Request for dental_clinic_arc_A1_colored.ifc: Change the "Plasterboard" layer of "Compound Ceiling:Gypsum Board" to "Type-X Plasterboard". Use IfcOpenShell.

First a look at what the model holds.

```python
import ifcopenshell
import ifcopenshell.util.element

model = ifcopenshell.open("dental_clinic_arc_A1_colored.ifc")
print(model.schema)
for layer_set in model.by_type("IfcMaterialLayerSet"):
    if layer_set.LayerSetName == "Compound Ceiling:Gypsum Board":
        for layer in layer_set.MaterialLayers:
            print(layer.id(), layer.Material and layer.Material.Name, layer.LayerThickness, sep=" | ")
        print(len(ifcopenshell.util.element.get_elements_by_material(model, layer_set)), "elements and types use it")
print(sorted(m.Name for m in model.by_type("IfcMaterial") if m.Name)[:60])
```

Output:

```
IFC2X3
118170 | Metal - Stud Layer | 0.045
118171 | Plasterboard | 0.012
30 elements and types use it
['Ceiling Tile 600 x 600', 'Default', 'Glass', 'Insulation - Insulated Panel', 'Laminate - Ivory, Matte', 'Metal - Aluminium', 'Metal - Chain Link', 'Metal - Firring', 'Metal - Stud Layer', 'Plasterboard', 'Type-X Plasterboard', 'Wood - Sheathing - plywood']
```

```python
import ifcopenshell
import ifcopenshell.api.material

model = ifcopenshell.open("dental_clinic_arc_A1_colored.ifc")

layer_set = next(s for s in model.by_type("IfcMaterialLayerSet") if s.LayerSetName == "Compound Ceiling:Gypsum Board")
layer = next(l for l in layer_set.MaterialLayers if l.Material and l.Material.Name == "Plasterboard")
material = next(m for m in model.by_type("IfcMaterial") if m.Name == "Type-X Plasterboard")

# Point this one layer at the other material; renaming the old one would change it everywhere.
ifcopenshell.api.material.edit_layer(model, layer=layer, attributes={}, material=material)

print([l.Material.Name if l.Material else None for l in layer_set.MaterialLayers])

model.write("dental_clinic_arc_A1_colored_edited.ifc")
```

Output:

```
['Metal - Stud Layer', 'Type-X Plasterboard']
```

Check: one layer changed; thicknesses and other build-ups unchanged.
